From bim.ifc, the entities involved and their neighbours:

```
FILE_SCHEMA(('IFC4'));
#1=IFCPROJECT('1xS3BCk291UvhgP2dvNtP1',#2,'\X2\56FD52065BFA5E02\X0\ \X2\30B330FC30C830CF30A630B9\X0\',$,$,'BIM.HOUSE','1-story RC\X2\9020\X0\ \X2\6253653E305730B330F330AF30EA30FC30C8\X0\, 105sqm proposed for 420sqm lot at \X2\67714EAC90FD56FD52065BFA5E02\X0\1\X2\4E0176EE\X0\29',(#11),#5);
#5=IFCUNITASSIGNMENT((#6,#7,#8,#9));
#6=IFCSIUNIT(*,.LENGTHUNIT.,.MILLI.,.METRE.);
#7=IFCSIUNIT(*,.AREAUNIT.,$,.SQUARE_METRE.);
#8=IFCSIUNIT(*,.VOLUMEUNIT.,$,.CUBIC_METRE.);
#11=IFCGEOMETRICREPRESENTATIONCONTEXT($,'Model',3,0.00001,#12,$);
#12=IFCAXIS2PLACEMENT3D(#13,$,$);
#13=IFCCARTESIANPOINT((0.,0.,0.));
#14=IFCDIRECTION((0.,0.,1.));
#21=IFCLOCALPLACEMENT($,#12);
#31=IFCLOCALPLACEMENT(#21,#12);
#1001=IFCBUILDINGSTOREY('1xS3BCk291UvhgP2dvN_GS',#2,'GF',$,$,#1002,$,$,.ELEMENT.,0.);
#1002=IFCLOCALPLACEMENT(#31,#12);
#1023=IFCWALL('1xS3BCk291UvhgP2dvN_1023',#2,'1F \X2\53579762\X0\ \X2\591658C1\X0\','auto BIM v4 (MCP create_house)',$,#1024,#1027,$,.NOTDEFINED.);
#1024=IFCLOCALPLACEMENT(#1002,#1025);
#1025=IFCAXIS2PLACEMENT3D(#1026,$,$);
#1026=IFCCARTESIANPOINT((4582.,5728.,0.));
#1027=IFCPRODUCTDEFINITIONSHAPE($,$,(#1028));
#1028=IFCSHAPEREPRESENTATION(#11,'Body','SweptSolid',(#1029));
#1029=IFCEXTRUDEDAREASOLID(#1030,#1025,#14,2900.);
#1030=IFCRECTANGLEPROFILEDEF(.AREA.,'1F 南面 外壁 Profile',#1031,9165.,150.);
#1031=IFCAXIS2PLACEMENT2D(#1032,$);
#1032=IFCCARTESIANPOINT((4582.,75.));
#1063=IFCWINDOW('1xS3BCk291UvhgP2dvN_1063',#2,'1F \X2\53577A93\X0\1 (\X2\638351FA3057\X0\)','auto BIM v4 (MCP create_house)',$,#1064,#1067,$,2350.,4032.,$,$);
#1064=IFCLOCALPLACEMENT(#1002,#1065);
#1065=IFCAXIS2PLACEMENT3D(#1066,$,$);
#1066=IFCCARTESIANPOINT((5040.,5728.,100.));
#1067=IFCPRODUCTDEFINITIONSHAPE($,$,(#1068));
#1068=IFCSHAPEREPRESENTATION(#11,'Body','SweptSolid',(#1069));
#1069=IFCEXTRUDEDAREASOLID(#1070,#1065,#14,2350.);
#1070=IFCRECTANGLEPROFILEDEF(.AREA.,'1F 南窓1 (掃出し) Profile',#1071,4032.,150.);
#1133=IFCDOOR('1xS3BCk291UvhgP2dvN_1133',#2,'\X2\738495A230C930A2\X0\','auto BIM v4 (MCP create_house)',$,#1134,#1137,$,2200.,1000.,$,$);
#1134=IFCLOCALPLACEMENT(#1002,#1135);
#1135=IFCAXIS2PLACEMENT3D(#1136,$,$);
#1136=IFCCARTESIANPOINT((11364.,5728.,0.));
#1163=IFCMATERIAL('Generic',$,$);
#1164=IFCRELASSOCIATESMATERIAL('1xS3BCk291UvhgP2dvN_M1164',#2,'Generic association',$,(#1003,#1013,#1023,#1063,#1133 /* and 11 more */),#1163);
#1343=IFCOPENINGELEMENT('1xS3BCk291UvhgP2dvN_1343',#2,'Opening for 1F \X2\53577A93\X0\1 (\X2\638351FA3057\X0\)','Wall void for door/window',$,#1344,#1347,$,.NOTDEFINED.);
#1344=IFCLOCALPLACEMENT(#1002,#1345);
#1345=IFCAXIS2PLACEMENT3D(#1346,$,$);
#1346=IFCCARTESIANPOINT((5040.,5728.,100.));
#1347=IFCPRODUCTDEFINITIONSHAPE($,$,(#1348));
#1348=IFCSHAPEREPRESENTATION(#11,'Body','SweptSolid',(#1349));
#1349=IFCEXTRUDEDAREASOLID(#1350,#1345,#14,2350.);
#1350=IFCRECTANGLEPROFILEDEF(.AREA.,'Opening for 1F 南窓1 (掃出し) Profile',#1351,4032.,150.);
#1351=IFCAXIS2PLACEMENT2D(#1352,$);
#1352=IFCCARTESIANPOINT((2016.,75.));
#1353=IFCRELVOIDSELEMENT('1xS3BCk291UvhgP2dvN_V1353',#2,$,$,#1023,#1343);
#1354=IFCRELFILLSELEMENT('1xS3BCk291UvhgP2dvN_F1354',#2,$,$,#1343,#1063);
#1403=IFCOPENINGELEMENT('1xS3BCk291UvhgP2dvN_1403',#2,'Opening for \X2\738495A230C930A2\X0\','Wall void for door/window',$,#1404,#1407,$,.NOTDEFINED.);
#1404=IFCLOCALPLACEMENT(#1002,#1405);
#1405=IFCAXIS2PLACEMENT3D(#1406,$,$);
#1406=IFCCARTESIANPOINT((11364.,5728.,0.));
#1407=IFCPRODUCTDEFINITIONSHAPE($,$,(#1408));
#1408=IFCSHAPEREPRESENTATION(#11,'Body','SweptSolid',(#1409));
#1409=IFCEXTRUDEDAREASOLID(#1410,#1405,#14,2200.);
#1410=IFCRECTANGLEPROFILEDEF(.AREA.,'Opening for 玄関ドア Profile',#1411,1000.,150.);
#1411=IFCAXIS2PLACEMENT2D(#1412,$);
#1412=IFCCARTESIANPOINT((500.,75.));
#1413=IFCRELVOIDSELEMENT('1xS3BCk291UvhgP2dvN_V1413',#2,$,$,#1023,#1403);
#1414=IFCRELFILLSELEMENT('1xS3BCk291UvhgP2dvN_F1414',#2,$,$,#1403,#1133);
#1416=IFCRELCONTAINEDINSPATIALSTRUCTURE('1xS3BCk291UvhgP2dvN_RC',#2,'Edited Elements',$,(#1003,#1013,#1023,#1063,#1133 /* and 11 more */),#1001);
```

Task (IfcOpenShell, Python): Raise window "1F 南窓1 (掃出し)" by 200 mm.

```python
import numpy as np
import ifcopenshell
import ifcopenshell.api.geometry
import ifcopenshell.util.placement
import ifcopenshell.util.unit

model = ifcopenshell.open("bim.ifc")
unit_scale = ifcopenshell.util.unit.calculate_unit_scale(model)

window = model.by_guid("1xS3BCk291UvhgP2dvN_1063")
opening = window.FillsVoids[0].RelatingOpeningElement
dz = 200.0

shift = np.array([0.0, 0.0, dz])
# The window is not placed relative to its opening, so move both.
for product in (opening, window):
    matrix = ifcopenshell.util.placement.get_local_placement(product.ObjectPlacement)
    matrix[:3, 3] += shift
    ifcopenshell.api.geometry.edit_object_placement(model, product=product, matrix=matrix, is_si=False)

print(f"moved by {dz * unit_scale:+.3f} m")

model.write("bim-out.ifc")
```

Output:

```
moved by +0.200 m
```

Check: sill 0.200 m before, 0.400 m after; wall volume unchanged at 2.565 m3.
